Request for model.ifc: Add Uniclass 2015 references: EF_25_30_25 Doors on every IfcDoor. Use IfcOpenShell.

First a look at what the model holds.

```python
import ifcopenshell

model = ifcopenshell.open("model.ifc")
print(model.schema)
print("classifications:", [c.Name for c in model.by_type("IfcClassification")])
for ifc_class in ("IfcDoor", "IfcRoof", "IfcStair", "IfcWall", "IfcWindow"):
    print(ifc_class, len(model.by_type(ifc_class)))
```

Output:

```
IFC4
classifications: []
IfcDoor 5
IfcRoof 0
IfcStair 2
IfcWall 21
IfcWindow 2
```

```python
import ifcopenshell
import ifcopenshell.api.classification

model = ifcopenshell.open("model.ifc")

system = ifcopenshell.api.classification.add_classification(model, classification="Uniclass 2015")

codes = {
    "IfcDoor": ("EF_25_30_25", "Doors"),
}
for ifc_class, (code, name) in codes.items():
    products = model.by_type(ifc_class)
    ifcopenshell.api.classification.add_reference(
        model, products=products, classification=system, identification=code, name=name
    )
    print(code, len(products))

model.write("model-out.ifc")
```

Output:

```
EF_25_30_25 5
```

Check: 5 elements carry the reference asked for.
